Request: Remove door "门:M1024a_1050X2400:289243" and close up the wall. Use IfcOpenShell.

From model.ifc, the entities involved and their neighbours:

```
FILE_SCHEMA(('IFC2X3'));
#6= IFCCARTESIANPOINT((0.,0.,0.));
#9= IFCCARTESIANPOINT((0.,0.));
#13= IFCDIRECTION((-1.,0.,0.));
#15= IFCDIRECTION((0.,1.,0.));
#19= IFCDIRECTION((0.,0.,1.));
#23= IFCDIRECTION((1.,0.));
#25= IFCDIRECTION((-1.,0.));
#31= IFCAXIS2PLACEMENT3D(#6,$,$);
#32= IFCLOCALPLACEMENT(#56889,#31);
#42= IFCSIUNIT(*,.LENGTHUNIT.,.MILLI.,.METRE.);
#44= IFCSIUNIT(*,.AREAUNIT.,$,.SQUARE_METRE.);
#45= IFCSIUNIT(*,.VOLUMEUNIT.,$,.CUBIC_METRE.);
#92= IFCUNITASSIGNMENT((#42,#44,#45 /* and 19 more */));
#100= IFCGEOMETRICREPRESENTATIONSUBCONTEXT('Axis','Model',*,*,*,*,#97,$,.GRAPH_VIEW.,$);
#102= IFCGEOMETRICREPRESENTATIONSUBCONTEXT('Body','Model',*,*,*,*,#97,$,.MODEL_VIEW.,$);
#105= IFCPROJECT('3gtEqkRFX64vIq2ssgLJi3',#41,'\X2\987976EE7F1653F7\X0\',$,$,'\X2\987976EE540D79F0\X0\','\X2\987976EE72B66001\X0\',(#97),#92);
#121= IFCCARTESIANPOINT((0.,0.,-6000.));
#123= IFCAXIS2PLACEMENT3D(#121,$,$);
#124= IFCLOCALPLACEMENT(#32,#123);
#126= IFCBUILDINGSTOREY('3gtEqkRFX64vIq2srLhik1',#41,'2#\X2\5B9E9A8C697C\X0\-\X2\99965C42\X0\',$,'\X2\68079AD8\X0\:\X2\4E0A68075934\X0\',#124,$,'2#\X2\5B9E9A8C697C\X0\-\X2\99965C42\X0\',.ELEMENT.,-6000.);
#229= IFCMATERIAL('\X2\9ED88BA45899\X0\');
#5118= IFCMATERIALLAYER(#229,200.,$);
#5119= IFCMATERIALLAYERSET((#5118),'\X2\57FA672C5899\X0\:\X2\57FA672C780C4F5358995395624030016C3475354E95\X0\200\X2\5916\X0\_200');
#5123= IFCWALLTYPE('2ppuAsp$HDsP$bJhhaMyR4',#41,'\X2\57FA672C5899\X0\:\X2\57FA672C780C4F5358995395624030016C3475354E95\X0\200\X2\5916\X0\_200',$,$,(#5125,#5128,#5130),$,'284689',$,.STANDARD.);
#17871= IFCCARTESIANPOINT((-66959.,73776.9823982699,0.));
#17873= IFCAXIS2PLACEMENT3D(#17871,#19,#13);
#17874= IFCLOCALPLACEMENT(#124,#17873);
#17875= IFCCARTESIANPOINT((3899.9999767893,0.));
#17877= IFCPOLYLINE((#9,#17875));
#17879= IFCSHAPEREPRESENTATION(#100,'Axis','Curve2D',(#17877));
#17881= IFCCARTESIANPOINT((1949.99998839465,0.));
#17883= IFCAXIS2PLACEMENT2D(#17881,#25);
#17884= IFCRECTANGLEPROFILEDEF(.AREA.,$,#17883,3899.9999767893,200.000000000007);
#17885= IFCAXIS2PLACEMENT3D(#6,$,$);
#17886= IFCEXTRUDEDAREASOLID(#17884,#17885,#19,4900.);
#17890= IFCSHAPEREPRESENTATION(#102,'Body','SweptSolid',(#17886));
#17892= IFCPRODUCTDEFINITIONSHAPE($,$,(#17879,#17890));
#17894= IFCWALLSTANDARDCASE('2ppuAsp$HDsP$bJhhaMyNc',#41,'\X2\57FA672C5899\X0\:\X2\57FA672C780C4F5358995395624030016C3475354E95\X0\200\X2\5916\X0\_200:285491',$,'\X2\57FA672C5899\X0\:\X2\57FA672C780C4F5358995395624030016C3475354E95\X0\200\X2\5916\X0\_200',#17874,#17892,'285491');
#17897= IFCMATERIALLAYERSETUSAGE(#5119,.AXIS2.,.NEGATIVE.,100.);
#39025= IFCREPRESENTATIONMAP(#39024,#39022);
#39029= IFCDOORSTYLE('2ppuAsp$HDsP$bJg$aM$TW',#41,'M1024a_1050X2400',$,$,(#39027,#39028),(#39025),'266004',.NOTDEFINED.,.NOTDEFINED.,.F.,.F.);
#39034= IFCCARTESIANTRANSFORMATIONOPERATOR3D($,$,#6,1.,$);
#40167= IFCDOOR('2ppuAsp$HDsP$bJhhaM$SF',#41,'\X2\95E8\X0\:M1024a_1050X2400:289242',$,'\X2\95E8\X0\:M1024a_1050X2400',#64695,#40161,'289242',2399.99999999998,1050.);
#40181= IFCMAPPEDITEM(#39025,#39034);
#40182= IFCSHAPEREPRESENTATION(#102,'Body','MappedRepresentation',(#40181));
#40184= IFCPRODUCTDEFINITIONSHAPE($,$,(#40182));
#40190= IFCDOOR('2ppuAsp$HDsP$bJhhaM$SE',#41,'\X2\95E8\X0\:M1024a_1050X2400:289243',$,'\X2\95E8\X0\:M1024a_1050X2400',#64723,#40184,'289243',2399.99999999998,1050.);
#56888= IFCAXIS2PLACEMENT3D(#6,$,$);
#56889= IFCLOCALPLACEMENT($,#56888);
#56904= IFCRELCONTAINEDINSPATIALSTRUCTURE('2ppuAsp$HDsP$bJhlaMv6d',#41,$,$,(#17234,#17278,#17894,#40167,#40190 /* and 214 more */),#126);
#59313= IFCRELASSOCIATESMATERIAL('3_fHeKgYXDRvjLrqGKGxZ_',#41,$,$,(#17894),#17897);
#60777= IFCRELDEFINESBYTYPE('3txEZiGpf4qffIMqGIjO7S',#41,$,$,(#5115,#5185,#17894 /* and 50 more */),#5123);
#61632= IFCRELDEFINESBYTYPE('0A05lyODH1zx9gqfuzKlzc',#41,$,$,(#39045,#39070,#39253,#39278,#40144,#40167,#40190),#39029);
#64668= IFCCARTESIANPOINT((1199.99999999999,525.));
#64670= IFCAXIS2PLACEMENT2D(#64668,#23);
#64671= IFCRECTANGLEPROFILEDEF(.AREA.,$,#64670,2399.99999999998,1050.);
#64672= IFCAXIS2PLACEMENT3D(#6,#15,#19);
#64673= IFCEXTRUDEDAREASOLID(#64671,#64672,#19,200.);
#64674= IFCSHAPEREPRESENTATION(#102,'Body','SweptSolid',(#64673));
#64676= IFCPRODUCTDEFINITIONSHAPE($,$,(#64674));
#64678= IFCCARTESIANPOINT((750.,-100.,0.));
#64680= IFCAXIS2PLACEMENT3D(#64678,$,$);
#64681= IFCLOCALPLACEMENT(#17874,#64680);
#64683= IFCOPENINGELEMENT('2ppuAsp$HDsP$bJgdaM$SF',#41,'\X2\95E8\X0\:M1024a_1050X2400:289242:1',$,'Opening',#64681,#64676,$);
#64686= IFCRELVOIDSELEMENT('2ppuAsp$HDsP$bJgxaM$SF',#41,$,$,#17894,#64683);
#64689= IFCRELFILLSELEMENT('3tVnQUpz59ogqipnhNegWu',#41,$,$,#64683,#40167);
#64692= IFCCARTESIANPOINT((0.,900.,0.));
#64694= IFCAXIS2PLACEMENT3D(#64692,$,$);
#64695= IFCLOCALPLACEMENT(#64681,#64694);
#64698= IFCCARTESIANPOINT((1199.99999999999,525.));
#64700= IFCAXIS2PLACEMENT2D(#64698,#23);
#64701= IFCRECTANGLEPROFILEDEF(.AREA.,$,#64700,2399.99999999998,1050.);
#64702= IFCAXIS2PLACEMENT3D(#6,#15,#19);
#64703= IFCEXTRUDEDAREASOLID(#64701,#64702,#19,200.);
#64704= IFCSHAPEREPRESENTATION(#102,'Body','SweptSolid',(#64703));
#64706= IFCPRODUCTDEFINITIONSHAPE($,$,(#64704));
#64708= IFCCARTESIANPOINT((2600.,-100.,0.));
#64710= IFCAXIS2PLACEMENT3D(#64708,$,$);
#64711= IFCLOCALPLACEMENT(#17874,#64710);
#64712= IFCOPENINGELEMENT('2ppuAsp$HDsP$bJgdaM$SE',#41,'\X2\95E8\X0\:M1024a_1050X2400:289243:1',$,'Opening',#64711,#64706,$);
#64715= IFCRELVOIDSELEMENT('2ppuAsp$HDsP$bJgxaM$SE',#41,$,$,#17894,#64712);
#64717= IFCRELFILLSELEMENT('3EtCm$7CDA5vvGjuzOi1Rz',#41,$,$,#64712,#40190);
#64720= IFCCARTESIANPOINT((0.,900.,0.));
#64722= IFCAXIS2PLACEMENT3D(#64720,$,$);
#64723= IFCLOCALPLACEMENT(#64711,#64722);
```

```python
import ifcopenshell
import ifcopenshell.api.feature
import ifcopenshell.api.root
import ifcopenshell.geom
import ifcopenshell.util.shape

model = ifcopenshell.open("model.ifc")
settings = ifcopenshell.geom.settings()


def volume(element):
    """Net volume in cubic metres, openings subtracted."""
    shape = ifcopenshell.geom.create_shape(settings, element)
    return ifcopenshell.util.shape.get_volume(shape.geometry)


door = model.by_guid("2ppuAsp$HDsP$bJhhaM$SE")
opening = door.FillsVoids[0].RelatingOpeningElement
wall = opening.VoidsElements[0].RelatingBuildingElement
before = volume(wall)

ifcopenshell.api.root.remove_product(model, product=door)
ifcopenshell.api.feature.remove_feature(model, feature=opening)

after = volume(wall)

print(f"wall volume {before:.3f} -> {after:.3f} m3")

model.write("model_updated.ifc")
```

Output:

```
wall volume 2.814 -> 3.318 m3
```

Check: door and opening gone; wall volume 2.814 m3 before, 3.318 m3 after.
